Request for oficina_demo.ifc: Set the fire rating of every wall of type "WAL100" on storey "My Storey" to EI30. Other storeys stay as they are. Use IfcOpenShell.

First a look at what the model holds.

```python
import ifcopenshell
import ifcopenshell.util.element

model = ifcopenshell.open("oficina_demo.ifc")
print(model.schema)
storey = next(s for s in model.by_type("IfcBuildingStorey") if s.Name == "My Storey")
walls = [e for e in ifcopenshell.util.element.get_decomposition(storey) if e.is_a("IfcWall")]
seen = {}
for e in walls:
    element_type = ifcopenshell.util.element.get_type(e)
    key = (element_type.Name if element_type != e and element_type else None, ifcopenshell.util.element.get_pset(e, "Pset_WallCommon", "FireRating"))
    seen[key] = seen.get(key, 0) + 1
for (name, value), count in sorted(seen.items(), key=str):
    print(count, "x", name, "|", value)
```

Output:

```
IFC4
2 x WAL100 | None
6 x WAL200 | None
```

```python
import ifcopenshell
import ifcopenshell.api.pset
import ifcopenshell.util.element

model = ifcopenshell.open("oficina_demo.ifc")

storey = next(s for s in model.by_type("IfcBuildingStorey") if s.Name == "My Storey")
walls = [e for e in ifcopenshell.util.element.get_decomposition(storey) if e.is_a("IfcWall")]

count = 0
for e in walls:
    element_type = ifcopenshell.util.element.get_type(e)
    if element_type in (None, e) or element_type.Name != "WAL100":
        continue
    # add_pset returns the element's existing set when there is one.
    pset = ifcopenshell.api.pset.add_pset(model, product=e, name="Pset_WallCommon")
    ifcopenshell.api.pset.edit_pset(model, pset=pset, properties={"FireRating": "EI30"})
    count += 1

print(count, "walls updated")

model.write("oficina_demo_v2.ifc")
```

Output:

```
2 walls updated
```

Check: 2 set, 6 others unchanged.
